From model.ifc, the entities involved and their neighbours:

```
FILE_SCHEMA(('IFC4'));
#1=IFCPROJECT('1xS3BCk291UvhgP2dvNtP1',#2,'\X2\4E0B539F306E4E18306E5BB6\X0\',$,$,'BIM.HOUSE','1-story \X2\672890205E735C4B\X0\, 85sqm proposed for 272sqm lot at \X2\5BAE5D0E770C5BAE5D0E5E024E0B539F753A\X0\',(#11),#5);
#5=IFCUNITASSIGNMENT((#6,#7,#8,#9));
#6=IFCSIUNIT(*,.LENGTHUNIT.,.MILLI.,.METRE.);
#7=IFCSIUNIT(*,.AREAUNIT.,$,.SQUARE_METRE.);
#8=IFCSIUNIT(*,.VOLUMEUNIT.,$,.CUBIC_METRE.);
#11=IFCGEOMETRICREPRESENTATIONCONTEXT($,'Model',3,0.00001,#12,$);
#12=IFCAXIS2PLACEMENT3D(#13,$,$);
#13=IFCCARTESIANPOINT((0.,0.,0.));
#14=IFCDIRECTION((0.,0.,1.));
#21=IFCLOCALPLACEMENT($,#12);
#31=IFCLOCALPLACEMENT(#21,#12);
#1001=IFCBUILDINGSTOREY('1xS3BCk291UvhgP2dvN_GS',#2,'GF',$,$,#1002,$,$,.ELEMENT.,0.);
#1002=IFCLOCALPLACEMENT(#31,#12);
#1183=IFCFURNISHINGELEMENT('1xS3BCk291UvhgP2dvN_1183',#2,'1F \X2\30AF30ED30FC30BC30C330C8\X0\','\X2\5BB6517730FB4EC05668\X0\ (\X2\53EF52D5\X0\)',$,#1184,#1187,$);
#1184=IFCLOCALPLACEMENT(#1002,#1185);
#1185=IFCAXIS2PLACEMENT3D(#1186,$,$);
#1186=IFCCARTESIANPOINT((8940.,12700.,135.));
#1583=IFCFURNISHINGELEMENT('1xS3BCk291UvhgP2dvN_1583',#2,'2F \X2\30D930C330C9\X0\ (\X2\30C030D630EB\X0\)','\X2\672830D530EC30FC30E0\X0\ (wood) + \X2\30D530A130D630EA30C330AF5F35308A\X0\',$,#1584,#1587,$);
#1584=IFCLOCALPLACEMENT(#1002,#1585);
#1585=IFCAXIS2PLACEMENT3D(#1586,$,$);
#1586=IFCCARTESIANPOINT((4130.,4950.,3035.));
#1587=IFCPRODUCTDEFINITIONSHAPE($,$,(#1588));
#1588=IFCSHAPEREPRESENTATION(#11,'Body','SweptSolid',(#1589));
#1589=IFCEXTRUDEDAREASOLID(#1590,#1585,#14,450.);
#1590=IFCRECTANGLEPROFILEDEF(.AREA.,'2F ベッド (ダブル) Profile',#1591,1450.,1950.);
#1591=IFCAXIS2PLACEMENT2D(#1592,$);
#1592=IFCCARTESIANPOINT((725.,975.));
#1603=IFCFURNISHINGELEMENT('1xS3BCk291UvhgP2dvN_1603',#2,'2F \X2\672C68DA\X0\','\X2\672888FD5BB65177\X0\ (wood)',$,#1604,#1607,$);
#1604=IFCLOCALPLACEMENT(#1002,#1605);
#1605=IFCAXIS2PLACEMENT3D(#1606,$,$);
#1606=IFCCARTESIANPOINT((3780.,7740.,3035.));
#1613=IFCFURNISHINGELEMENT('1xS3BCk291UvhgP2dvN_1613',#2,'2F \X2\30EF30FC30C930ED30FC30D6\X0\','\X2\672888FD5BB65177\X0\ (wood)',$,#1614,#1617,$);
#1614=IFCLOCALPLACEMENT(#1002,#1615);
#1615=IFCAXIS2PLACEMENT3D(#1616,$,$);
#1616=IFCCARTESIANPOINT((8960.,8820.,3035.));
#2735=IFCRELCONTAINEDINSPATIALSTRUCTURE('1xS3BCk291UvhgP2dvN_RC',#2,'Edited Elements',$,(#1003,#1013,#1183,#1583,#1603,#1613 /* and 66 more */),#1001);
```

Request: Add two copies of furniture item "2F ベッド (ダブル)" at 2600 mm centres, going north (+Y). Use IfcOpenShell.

```python
import numpy as np
import ifcopenshell
import ifcopenshell.api.geometry
import ifcopenshell.api.root
import ifcopenshell.util.element
import ifcopenshell.util.placement
import ifcopenshell.util.unit

model = ifcopenshell.open("model.ifc")
unit_scale = ifcopenshell.util.unit.calculate_unit_scale(model)


def reuse_history(source, copy):
    """copy_class also copies each property set's owner history, people and application; keep the originals."""
    for rel in copy.IsDefinedBy:
        if rel.is_a("IfcRelDefinesByProperties") and (history := rel.RelatingPropertyDefinition.OwnerHistory):
            rel.RelatingPropertyDefinition.OwnerHistory = source.OwnerHistory
            ifcopenshell.util.element.remove_deep2(model, history)


source = model.by_guid("1xS3BCk291UvhgP2dvN_1583")
base = ifcopenshell.util.placement.get_local_placement(source.ObjectPlacement)
step = np.array([0.0, 1.0, 0.0]) * 2.6 / unit_scale

for i in range(1, 3):
    copy = ifcopenshell.api.root.copy_class(model, product=source)
    copy.Representation = ifcopenshell.util.element.copy_deep(
        model, source.Representation, exclude=["IfcGeometricRepresentationContext", "IfcRepresentationMap"]
    )
    reuse_history(source, copy)
    matrix = base.copy()
    matrix[:3, 3] += i * step
    print("added at", matrix[:3, 3].round(3) + 0.0)
    ifcopenshell.api.geometry.edit_object_placement(model, product=copy, matrix=matrix, is_si=False)

model.write("model_updated.ifc")
```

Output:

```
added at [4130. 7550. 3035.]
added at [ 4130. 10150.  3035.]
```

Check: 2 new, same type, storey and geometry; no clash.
